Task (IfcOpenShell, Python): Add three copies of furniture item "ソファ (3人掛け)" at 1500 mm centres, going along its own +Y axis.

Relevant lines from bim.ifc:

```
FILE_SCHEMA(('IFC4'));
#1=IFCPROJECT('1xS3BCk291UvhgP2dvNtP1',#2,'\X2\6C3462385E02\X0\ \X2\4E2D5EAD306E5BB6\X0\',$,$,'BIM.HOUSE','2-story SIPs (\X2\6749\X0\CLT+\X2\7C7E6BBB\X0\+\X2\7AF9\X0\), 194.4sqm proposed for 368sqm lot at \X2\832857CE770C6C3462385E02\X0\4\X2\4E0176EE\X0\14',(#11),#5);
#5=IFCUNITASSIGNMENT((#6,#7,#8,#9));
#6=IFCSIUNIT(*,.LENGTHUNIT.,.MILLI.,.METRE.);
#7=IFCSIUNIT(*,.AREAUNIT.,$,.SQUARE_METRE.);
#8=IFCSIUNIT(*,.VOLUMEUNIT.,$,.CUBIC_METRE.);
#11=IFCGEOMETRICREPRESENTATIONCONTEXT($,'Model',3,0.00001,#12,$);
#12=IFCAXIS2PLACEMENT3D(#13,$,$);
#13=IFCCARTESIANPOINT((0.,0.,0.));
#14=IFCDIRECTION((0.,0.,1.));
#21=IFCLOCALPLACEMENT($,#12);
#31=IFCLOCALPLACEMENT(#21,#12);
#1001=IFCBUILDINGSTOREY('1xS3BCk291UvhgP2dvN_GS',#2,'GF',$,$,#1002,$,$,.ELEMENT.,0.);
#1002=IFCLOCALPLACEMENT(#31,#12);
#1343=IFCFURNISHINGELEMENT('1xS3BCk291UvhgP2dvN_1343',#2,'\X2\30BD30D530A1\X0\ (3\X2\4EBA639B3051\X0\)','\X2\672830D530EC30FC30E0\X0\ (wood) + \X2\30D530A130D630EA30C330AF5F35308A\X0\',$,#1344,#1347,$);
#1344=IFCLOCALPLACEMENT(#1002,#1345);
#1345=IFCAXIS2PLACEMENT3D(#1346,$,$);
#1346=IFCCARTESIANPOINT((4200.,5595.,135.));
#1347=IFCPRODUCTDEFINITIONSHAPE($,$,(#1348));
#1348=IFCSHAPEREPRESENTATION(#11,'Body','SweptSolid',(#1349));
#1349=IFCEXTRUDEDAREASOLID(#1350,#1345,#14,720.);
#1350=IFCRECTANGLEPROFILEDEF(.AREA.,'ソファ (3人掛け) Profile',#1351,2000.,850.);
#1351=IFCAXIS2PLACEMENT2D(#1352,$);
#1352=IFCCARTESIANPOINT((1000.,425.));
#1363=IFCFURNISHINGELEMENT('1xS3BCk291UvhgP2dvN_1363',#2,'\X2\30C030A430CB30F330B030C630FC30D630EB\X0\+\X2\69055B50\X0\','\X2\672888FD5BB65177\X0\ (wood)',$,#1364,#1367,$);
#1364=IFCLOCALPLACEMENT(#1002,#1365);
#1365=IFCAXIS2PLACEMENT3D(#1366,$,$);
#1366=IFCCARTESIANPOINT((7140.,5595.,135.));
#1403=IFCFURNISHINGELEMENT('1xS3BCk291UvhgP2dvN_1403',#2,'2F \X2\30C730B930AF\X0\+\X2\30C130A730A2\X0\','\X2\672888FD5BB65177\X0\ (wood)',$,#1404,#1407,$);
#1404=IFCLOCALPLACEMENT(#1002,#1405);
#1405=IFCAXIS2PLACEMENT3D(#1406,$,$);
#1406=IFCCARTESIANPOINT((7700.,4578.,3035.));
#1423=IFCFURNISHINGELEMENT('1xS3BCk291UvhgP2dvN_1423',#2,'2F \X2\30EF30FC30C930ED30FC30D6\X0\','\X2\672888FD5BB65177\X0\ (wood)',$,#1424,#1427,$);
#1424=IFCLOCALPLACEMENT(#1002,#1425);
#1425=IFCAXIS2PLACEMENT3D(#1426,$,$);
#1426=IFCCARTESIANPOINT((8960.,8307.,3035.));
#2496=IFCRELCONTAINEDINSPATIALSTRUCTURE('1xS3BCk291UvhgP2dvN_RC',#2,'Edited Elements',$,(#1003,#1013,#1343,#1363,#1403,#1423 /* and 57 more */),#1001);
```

```python
import ifcopenshell
import ifcopenshell.api.geometry
import ifcopenshell.api.root
import ifcopenshell.util.element
import ifcopenshell.util.placement

model = ifcopenshell.open("bim.ifc")


def reuse_history(source, copy):
    """copy_class also copies each property set's owner history, people and application; keep the originals."""
    for rel in copy.IsDefinedBy:
        if rel.is_a("IfcRelDefinesByProperties") and (history := rel.RelatingPropertyDefinition.OwnerHistory):
            rel.RelatingPropertyDefinition.OwnerHistory = source.OwnerHistory
            ifcopenshell.util.element.remove_deep2(model, history)


source = model.by_guid("1xS3BCk291UvhgP2dvN_1343")
base = ifcopenshell.util.placement.get_local_placement(source.ObjectPlacement)
step = base[:3, 1] * 1500.0

for i in range(1, 4):
    copy = ifcopenshell.api.root.copy_class(model, product=source)
    copy.Representation = ifcopenshell.util.element.copy_deep(
        model, source.Representation, exclude=["IfcGeometricRepresentationContext", "IfcRepresentationMap"]
    )
    reuse_history(source, copy)
    matrix = base.copy()
    matrix[:3, 3] += i * step
    print("added at", matrix[:3, 3].round(3) + 0.0)
    ifcopenshell.api.geometry.edit_object_placement(model, product=copy, matrix=matrix, is_si=False)

model.write("bim_edited.ifc")
```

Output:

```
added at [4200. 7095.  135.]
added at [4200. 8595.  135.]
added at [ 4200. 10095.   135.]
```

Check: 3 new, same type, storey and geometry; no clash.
